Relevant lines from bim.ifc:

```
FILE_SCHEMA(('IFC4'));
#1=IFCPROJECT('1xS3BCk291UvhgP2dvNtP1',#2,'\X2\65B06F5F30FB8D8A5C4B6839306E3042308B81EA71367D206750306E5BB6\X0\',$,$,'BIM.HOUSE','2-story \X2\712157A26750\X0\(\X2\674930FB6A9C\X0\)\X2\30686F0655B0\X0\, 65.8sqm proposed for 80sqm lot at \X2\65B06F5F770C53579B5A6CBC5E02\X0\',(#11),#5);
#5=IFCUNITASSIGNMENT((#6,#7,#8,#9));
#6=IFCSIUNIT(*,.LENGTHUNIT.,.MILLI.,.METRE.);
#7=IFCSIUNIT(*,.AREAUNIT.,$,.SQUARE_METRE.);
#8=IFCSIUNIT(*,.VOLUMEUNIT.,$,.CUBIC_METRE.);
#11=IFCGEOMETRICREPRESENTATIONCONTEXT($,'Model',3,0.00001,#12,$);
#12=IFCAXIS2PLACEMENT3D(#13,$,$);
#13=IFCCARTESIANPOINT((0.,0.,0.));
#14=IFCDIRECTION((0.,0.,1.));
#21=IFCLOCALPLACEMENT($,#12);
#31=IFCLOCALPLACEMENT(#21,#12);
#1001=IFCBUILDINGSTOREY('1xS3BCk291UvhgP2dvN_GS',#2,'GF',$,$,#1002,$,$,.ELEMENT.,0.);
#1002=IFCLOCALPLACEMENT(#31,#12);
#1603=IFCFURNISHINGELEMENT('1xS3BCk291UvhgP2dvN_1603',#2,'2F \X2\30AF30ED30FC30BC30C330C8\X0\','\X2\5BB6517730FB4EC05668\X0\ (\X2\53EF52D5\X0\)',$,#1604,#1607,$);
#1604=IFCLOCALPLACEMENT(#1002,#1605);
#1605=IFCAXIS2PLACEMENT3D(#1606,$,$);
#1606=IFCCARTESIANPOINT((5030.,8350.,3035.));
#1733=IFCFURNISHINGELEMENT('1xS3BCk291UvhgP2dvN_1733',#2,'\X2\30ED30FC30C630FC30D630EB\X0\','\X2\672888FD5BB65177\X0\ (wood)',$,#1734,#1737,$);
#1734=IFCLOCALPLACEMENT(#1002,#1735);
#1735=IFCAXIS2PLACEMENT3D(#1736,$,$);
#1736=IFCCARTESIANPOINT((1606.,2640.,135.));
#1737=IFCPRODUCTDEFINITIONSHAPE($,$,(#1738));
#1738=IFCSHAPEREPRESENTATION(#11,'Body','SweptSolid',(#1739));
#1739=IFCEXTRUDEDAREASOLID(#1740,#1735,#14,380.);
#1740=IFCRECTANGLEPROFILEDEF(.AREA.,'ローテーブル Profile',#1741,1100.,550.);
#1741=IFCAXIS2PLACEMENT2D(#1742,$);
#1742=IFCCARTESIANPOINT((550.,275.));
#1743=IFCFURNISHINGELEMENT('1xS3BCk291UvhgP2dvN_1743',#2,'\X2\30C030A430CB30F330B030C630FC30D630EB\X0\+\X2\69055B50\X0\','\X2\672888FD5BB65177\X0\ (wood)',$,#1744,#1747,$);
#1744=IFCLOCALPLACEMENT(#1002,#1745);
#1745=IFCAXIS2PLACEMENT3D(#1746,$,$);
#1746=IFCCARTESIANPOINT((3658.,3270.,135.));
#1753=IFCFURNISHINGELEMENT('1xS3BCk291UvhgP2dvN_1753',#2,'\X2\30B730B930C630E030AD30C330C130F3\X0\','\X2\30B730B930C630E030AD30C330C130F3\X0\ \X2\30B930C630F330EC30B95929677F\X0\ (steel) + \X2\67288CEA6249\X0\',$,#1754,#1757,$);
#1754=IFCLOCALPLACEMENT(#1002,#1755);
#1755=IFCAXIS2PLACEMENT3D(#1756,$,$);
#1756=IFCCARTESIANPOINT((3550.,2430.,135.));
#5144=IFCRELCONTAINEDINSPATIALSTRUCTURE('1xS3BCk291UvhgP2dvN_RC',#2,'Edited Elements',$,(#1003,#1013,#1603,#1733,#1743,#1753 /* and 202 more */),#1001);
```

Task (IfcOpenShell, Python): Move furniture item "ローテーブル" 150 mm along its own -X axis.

```python
import ifcopenshell
import ifcopenshell.api.geometry
import ifcopenshell.util.placement
import ifcopenshell.util.unit

model = ifcopenshell.open("bim.ifc")
unit_scale = ifcopenshell.util.unit.calculate_unit_scale(model)

item = model.by_guid("1xS3BCk291UvhgP2dvN_1733")
matrix = ifcopenshell.util.placement.get_local_placement(item.ObjectPlacement)
matrix[:3, 3] -= matrix[:3, 0] * 0.15 / unit_scale
ifcopenshell.api.geometry.edit_object_placement(model, product=item, matrix=matrix, is_si=False)

print(ifcopenshell.util.placement.get_local_placement(item.ObjectPlacement).round(3) + 0.0)

model.write("bim-out.ifc")
```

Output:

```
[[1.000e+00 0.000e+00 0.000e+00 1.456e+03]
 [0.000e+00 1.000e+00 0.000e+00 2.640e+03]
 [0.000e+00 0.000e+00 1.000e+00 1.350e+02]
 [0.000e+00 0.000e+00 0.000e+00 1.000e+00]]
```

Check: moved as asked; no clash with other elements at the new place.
